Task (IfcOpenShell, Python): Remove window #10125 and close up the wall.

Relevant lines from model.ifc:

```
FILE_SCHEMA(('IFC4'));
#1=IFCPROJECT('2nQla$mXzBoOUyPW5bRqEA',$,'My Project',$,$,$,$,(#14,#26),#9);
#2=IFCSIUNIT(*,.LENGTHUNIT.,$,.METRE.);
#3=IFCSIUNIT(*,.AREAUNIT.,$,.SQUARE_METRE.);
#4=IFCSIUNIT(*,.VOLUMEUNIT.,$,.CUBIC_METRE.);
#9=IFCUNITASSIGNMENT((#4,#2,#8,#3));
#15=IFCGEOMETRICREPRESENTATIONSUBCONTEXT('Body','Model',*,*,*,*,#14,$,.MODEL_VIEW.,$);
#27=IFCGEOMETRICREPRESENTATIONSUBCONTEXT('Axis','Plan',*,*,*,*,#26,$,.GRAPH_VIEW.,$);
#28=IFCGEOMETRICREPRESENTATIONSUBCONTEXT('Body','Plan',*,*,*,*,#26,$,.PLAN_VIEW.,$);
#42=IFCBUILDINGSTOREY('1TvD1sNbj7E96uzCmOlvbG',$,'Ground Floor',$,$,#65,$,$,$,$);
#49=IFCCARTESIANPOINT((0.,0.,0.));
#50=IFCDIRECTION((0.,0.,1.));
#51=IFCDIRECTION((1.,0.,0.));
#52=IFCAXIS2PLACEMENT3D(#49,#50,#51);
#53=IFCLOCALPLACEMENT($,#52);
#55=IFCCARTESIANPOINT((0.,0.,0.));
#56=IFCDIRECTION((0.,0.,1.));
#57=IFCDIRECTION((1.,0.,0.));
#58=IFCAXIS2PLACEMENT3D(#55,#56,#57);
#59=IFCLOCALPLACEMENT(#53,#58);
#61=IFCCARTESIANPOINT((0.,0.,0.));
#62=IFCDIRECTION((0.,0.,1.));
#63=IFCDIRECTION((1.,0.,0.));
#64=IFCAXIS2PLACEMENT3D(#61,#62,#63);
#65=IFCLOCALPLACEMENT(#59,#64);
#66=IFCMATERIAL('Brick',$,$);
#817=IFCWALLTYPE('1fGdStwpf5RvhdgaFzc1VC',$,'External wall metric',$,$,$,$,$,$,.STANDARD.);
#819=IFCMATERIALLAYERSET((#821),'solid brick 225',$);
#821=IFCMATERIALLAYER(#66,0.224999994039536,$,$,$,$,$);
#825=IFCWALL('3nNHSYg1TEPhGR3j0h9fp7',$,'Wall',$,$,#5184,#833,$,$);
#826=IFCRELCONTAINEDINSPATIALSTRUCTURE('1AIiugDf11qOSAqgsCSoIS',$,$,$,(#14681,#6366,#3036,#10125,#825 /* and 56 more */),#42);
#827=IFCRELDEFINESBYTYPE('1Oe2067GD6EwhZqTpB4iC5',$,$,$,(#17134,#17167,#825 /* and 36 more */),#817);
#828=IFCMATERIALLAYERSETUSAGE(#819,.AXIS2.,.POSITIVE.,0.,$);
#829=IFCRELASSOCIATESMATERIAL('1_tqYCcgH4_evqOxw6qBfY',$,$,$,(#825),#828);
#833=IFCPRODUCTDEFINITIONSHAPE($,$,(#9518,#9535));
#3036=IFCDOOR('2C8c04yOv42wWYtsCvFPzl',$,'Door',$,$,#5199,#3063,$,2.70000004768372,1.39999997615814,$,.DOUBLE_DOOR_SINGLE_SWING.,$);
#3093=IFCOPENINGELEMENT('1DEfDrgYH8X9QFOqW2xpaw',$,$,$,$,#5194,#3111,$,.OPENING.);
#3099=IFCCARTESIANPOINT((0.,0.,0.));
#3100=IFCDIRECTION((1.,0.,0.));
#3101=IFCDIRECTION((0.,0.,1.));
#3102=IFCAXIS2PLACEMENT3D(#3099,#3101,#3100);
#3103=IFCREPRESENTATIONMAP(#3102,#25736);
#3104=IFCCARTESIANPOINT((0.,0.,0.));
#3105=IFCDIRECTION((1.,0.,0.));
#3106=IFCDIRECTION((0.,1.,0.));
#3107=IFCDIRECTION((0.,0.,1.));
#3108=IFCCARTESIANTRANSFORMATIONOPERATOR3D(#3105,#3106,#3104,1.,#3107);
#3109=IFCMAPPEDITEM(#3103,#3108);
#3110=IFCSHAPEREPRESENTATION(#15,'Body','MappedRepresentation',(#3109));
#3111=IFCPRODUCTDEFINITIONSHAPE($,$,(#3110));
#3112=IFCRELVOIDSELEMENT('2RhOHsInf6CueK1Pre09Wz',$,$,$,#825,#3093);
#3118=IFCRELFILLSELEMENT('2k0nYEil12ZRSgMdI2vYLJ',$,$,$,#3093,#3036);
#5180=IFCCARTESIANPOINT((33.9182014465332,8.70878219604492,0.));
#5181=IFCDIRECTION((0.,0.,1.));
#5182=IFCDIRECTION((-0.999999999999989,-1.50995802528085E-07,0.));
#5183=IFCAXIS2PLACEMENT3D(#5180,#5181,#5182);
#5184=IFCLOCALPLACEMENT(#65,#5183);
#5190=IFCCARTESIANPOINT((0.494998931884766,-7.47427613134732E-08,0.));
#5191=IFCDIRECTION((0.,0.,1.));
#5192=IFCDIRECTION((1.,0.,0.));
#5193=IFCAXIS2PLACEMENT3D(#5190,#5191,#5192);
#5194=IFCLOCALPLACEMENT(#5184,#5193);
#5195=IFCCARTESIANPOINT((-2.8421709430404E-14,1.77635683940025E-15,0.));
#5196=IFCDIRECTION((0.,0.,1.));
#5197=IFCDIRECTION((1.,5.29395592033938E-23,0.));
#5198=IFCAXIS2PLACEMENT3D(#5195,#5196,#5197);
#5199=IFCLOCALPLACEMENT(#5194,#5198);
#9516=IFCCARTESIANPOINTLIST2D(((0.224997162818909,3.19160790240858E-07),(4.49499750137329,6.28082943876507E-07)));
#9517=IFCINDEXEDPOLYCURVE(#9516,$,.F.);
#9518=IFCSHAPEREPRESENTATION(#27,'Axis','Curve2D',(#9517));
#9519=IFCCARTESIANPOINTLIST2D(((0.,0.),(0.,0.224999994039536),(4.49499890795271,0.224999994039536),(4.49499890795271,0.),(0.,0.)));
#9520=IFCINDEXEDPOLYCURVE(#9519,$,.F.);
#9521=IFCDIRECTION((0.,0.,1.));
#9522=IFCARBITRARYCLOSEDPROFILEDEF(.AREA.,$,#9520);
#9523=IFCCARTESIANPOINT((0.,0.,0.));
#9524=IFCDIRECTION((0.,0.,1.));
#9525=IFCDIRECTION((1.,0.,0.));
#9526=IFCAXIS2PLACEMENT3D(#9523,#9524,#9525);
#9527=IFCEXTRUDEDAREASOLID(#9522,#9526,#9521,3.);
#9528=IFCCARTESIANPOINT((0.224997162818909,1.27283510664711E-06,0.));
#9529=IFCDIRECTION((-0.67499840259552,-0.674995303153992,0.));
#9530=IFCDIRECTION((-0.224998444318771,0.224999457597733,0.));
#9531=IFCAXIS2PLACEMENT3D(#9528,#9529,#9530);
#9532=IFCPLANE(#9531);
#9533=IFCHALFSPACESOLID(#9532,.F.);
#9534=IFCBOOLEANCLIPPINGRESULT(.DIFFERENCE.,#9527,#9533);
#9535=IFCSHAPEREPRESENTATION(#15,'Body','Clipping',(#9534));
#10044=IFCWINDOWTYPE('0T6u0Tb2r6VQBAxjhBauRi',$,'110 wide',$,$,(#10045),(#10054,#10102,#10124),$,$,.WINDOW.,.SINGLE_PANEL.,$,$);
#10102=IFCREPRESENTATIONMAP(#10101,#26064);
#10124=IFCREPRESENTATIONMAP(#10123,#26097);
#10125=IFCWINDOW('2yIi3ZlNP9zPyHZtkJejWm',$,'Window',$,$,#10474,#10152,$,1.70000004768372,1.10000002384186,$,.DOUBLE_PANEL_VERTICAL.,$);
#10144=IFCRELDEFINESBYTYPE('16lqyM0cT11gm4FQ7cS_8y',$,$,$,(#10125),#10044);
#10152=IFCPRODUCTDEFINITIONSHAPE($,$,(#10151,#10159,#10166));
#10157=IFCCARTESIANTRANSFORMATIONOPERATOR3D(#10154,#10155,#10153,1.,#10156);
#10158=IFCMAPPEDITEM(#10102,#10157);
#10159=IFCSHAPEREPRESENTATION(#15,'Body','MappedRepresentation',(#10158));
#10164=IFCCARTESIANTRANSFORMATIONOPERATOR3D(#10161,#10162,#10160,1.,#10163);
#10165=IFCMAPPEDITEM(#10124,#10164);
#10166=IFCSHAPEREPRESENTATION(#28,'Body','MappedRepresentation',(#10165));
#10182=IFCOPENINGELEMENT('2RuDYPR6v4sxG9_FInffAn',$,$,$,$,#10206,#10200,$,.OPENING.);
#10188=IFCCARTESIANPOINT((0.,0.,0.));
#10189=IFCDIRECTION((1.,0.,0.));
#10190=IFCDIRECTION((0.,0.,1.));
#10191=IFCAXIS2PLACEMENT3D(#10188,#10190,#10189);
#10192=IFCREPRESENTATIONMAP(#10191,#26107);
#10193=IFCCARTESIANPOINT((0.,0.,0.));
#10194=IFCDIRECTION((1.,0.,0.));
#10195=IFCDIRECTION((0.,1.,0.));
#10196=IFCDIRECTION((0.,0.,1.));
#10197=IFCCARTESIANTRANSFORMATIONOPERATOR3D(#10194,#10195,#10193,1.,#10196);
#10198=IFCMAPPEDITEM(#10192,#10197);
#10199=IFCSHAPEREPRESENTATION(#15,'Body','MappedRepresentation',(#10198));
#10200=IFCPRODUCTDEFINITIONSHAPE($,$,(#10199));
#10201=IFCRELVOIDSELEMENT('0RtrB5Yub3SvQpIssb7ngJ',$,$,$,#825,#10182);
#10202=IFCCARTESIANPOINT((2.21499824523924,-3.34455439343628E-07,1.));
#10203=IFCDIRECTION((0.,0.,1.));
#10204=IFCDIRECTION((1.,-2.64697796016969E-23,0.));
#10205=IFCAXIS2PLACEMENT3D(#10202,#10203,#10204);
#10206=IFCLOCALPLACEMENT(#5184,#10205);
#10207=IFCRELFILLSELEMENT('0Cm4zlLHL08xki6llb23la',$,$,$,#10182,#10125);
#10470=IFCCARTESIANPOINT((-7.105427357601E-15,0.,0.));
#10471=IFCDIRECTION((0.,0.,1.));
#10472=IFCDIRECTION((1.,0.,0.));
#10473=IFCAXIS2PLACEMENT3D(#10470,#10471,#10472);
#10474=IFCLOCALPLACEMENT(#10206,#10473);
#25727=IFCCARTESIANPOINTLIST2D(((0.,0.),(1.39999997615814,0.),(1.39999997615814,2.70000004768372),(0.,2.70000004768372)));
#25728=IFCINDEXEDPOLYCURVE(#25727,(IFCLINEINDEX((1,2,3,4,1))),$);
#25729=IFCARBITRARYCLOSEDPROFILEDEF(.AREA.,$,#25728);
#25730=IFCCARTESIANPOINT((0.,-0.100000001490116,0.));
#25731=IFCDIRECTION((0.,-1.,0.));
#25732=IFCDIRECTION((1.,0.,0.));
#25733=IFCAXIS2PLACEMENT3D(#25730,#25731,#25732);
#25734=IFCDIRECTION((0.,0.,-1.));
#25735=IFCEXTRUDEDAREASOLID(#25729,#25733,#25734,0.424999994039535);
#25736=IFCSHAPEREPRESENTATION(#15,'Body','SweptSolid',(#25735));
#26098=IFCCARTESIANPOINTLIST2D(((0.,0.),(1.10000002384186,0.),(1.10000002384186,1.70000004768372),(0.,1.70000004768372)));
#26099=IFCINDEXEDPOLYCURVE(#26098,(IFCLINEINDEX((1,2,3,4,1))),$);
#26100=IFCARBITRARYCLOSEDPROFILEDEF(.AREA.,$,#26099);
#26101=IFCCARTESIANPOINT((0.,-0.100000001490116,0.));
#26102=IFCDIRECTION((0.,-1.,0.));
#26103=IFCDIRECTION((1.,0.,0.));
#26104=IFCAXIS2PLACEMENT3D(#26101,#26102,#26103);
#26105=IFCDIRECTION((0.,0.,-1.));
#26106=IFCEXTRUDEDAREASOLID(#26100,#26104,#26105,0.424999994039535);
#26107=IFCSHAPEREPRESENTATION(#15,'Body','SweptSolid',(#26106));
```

```python
import ifcopenshell
import ifcopenshell.api.feature
import ifcopenshell.api.root
import ifcopenshell.geom
import ifcopenshell.util.shape

model = ifcopenshell.open("model.ifc")
settings = ifcopenshell.geom.settings()


def volume(element):
    """Net volume in cubic metres, openings subtracted."""
    shape = ifcopenshell.geom.create_shape(settings, element)
    return ifcopenshell.util.shape.get_volume(shape.geometry)


window = model.by_guid("2yIi3ZlNP9zPyHZtkJejWm")
opening = window.FillsVoids[0].RelatingOpeningElement
wall = opening.VoidsElements[0].RelatingBuildingElement
before = volume(wall)

ifcopenshell.api.root.remove_product(model, product=window)
ifcopenshell.api.feature.remove_feature(model, feature=opening)

after = volume(wall)

print(f"wall volume {before:.3f} -> {after:.3f} m3")

model.write("model_updated.ifc")
```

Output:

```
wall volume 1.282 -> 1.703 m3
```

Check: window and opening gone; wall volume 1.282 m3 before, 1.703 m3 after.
